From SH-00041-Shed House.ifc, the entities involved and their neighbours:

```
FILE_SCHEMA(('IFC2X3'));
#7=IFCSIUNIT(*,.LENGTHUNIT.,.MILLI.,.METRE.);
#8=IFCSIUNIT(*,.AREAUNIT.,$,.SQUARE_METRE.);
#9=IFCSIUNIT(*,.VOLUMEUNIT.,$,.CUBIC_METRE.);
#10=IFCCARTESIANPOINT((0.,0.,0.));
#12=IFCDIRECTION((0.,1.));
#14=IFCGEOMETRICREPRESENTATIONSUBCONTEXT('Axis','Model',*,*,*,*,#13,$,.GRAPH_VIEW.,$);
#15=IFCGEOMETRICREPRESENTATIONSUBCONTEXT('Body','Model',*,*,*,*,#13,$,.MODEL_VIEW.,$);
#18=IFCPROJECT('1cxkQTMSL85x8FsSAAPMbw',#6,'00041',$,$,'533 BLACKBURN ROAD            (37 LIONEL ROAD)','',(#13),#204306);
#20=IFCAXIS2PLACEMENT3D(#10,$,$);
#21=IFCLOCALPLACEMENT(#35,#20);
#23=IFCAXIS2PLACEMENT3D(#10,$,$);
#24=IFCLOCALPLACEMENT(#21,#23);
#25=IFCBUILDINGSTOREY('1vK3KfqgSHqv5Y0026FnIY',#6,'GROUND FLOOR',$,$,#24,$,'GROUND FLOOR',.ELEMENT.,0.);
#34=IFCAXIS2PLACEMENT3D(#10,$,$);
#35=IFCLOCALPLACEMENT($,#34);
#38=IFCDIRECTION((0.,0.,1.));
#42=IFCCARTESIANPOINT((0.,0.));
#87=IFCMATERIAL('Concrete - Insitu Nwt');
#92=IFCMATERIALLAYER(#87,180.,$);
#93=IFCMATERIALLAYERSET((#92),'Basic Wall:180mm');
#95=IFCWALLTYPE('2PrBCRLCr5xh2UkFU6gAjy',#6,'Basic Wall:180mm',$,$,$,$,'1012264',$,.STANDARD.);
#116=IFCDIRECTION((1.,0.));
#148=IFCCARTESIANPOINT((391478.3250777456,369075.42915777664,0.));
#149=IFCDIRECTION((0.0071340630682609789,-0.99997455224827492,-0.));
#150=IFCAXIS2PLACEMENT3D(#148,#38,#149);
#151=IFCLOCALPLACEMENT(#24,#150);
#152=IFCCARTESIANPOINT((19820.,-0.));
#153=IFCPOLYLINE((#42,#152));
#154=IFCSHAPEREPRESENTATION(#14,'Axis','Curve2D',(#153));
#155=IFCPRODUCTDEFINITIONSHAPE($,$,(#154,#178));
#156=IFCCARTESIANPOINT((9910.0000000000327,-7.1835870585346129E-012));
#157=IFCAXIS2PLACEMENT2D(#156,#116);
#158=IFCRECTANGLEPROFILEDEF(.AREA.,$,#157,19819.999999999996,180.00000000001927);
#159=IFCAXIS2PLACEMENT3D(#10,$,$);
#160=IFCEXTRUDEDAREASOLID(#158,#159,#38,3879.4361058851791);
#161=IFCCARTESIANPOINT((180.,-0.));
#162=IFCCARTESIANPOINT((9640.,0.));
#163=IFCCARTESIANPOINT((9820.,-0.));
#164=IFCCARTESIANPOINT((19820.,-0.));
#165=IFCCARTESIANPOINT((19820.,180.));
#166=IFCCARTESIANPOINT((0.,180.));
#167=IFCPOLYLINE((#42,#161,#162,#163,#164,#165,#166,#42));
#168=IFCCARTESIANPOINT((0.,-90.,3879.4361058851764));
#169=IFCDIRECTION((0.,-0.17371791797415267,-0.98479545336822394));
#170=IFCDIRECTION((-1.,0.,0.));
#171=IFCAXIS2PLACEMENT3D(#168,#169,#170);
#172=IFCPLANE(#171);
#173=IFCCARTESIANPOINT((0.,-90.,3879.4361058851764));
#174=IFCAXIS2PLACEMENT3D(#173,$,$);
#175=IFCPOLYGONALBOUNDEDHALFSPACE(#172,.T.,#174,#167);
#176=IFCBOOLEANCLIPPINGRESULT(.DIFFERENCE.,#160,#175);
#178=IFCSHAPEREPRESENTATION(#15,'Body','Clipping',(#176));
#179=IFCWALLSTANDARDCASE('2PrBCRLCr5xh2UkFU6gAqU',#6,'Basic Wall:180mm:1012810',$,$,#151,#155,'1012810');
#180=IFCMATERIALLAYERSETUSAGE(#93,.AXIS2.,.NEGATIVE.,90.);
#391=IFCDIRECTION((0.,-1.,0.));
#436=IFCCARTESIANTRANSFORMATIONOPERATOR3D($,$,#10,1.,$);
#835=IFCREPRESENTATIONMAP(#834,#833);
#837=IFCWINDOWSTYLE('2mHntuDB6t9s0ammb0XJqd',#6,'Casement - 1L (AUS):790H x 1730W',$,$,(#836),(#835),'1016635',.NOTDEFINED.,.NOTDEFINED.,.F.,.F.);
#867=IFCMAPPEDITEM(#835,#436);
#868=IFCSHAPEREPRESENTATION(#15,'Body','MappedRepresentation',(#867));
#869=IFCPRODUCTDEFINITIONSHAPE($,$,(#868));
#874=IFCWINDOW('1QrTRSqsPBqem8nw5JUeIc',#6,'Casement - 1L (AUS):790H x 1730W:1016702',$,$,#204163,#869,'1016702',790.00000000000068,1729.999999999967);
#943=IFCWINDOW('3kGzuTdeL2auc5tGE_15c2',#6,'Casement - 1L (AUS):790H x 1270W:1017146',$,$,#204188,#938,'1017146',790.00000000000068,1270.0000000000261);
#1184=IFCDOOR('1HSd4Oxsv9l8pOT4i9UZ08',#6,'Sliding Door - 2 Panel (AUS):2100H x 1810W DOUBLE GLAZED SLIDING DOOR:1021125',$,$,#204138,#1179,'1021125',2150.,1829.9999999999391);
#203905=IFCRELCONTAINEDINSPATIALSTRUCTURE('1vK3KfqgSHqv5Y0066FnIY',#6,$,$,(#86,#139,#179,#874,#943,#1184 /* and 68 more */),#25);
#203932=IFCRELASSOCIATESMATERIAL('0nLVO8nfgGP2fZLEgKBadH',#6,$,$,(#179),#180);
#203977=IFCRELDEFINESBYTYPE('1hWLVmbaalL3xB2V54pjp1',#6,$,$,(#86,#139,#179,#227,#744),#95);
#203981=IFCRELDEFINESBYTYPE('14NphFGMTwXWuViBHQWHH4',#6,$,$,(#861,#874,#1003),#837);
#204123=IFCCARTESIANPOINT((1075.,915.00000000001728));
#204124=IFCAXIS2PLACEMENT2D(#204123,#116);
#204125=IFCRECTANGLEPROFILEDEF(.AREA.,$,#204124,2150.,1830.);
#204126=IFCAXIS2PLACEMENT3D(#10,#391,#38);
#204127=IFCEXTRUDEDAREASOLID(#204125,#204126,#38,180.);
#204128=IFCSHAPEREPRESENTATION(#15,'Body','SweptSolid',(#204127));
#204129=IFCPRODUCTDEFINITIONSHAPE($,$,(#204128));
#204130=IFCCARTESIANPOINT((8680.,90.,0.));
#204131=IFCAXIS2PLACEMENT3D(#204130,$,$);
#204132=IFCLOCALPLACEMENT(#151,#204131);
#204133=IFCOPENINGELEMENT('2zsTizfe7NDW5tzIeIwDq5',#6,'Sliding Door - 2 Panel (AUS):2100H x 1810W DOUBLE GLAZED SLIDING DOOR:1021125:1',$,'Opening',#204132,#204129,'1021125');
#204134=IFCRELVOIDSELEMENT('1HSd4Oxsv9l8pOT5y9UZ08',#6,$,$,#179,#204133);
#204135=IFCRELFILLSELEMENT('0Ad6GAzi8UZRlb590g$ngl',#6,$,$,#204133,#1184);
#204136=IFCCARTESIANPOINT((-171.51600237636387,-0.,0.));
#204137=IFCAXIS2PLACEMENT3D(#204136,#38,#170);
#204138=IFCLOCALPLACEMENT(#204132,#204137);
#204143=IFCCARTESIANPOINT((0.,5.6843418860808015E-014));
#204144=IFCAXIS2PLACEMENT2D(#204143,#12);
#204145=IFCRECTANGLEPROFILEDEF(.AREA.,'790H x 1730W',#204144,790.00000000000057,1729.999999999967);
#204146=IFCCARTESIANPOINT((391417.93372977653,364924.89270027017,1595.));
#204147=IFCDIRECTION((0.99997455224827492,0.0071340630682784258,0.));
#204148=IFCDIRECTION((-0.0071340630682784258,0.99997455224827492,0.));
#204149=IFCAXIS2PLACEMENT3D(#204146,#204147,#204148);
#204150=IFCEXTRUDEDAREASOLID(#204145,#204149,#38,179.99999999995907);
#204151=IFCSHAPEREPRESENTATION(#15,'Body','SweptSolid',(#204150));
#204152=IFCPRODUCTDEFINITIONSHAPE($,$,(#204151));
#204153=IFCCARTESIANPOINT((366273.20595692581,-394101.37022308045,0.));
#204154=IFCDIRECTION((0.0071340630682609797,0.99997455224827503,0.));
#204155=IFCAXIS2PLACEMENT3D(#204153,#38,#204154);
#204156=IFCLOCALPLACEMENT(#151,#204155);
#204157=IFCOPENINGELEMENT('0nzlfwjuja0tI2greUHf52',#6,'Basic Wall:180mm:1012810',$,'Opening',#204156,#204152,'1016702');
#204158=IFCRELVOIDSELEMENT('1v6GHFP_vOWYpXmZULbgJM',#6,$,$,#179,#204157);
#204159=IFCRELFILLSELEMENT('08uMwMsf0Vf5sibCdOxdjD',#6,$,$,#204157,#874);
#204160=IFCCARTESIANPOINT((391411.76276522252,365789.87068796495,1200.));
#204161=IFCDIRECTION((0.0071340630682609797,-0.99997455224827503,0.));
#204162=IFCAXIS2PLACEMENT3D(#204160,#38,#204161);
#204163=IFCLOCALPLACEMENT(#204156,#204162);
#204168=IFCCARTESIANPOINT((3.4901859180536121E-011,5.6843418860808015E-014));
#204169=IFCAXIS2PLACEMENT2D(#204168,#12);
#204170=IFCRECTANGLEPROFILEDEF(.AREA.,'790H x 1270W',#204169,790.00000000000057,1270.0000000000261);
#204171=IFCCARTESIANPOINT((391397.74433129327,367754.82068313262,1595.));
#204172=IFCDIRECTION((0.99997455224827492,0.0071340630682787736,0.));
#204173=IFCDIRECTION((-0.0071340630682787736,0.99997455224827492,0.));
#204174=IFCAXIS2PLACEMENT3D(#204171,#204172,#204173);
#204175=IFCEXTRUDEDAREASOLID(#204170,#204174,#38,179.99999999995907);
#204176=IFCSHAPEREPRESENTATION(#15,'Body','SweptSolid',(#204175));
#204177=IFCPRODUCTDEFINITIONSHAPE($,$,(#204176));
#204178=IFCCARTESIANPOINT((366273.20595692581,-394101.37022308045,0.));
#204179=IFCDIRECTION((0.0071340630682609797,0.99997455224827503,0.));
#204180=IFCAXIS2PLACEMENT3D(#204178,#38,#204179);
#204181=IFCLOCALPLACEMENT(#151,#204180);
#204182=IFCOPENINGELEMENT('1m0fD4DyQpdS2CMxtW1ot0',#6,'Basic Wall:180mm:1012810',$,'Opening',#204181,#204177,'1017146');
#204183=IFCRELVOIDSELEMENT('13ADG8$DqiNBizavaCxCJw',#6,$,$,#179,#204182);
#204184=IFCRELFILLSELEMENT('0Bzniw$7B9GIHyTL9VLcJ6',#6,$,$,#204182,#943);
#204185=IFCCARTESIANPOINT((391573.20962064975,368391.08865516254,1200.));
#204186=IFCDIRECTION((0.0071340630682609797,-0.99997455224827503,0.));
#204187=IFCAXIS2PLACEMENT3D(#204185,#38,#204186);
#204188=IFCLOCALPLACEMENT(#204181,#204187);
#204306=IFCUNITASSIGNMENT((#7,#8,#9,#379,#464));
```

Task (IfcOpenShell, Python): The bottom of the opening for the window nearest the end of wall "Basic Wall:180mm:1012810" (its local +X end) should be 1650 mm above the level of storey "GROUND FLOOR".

```python
import numpy as np
import ifcopenshell
import ifcopenshell.api.geometry
import ifcopenshell.geom
import ifcopenshell.util.element
import ifcopenshell.util.placement
import ifcopenshell.util.shape
import ifcopenshell.util.unit

model = ifcopenshell.open("SH-00041-Shed House.ifc")
unit_scale = ifcopenshell.util.unit.calculate_unit_scale(model)

window = model.by_id(874)
opening = window.FillsVoids[0].RelatingOpeningElement
storey = ifcopenshell.util.element.get_container(window, ifc_class="IfcBuildingStorey")
level = ifcopenshell.util.placement.get_local_placement(storey.ObjectPlacement)[2, 3]

# The opening's origin need not be at the sill, so measure its lowest point.
shape = ifcopenshell.geom.create_shape(ifcopenshell.geom.settings(), opening)
bottom = ifcopenshell.util.shape.get_shape_bottom_elevation(shape, shape.geometry) / unit_scale
dz = level + 1650.0 - bottom

shift = np.array([0.0, 0.0, dz])
# The window is placed relative to its opening, so it follows when the opening moves.
matrix = ifcopenshell.util.placement.get_local_placement(opening.ObjectPlacement)
matrix[:3, 3] += shift
ifcopenshell.api.geometry.edit_object_placement(
    model, product=opening, matrix=matrix, is_si=False, should_transform_children=True
)

print(f"moved by {dz * unit_scale:+.3f} m")

model.write("SH-00041-Shed House_updated.ifc")
```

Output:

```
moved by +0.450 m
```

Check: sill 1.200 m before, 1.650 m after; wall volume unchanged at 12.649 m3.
